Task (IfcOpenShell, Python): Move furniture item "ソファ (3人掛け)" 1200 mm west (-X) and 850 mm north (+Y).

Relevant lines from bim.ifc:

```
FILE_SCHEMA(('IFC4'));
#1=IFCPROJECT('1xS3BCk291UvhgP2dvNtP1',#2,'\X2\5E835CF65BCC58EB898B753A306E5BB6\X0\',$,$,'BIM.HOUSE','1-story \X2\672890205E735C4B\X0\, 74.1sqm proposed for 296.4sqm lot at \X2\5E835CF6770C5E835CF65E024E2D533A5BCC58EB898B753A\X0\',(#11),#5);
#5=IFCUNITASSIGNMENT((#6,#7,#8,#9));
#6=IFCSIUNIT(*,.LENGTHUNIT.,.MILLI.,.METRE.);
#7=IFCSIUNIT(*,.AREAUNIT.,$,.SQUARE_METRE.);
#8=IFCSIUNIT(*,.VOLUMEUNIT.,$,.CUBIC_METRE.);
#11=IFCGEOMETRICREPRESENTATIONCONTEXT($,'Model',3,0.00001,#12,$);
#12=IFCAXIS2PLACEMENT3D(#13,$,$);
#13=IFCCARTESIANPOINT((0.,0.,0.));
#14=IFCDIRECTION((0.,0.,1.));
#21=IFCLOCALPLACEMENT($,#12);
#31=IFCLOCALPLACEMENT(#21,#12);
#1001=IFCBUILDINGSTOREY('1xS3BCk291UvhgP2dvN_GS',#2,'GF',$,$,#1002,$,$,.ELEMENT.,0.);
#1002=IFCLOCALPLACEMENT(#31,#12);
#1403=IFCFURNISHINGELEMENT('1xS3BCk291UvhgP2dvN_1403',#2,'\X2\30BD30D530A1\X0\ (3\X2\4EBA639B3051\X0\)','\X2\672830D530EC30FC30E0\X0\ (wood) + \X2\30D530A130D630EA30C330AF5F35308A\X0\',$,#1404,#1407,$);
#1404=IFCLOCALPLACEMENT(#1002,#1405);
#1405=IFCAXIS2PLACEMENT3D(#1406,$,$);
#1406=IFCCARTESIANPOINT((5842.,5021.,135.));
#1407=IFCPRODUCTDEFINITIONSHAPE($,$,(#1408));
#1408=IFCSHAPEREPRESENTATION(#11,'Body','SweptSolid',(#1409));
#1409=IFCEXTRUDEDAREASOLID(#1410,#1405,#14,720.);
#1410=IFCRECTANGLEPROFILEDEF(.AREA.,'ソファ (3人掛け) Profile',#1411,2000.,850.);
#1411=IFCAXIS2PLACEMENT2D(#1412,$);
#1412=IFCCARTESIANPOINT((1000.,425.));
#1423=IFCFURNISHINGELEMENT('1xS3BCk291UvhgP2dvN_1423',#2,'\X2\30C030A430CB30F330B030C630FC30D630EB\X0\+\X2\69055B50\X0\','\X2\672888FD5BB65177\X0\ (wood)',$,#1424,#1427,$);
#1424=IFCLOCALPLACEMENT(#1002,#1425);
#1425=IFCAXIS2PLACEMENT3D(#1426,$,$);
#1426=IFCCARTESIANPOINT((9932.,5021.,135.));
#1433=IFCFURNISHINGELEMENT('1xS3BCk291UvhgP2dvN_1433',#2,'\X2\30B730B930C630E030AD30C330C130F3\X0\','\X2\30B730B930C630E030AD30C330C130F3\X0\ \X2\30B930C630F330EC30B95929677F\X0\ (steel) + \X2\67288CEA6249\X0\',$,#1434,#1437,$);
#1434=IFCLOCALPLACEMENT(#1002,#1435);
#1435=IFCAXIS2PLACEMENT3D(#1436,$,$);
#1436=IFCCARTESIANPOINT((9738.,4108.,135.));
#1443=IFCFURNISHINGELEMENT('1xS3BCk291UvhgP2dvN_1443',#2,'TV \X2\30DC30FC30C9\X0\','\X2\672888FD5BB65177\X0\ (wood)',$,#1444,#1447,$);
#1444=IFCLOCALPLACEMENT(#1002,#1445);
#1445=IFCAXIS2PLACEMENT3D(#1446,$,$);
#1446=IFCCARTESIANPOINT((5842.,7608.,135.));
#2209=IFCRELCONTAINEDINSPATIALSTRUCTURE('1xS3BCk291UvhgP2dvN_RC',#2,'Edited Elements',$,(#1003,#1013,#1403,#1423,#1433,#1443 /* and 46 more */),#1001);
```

```python
import ifcopenshell
import ifcopenshell.api.geometry
import ifcopenshell.util.placement
import ifcopenshell.util.unit

model = ifcopenshell.open("bim.ifc")
unit_scale = ifcopenshell.util.unit.calculate_unit_scale(model)

item = model.by_guid("1xS3BCk291UvhgP2dvN_1403")
matrix = ifcopenshell.util.placement.get_local_placement(item.ObjectPlacement)
matrix[0, 3] -= 1.2 / unit_scale
matrix[1, 3] += 0.85 / unit_scale
ifcopenshell.api.geometry.edit_object_placement(model, product=item, matrix=matrix, is_si=False)

print(ifcopenshell.util.placement.get_local_placement(item.ObjectPlacement).round(3) + 0.0)

model.write("bim_rev.ifc")
```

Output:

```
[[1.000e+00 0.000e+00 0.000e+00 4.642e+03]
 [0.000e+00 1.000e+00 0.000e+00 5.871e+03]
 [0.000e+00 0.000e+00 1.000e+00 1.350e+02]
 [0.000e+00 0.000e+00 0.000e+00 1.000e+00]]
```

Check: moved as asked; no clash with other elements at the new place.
